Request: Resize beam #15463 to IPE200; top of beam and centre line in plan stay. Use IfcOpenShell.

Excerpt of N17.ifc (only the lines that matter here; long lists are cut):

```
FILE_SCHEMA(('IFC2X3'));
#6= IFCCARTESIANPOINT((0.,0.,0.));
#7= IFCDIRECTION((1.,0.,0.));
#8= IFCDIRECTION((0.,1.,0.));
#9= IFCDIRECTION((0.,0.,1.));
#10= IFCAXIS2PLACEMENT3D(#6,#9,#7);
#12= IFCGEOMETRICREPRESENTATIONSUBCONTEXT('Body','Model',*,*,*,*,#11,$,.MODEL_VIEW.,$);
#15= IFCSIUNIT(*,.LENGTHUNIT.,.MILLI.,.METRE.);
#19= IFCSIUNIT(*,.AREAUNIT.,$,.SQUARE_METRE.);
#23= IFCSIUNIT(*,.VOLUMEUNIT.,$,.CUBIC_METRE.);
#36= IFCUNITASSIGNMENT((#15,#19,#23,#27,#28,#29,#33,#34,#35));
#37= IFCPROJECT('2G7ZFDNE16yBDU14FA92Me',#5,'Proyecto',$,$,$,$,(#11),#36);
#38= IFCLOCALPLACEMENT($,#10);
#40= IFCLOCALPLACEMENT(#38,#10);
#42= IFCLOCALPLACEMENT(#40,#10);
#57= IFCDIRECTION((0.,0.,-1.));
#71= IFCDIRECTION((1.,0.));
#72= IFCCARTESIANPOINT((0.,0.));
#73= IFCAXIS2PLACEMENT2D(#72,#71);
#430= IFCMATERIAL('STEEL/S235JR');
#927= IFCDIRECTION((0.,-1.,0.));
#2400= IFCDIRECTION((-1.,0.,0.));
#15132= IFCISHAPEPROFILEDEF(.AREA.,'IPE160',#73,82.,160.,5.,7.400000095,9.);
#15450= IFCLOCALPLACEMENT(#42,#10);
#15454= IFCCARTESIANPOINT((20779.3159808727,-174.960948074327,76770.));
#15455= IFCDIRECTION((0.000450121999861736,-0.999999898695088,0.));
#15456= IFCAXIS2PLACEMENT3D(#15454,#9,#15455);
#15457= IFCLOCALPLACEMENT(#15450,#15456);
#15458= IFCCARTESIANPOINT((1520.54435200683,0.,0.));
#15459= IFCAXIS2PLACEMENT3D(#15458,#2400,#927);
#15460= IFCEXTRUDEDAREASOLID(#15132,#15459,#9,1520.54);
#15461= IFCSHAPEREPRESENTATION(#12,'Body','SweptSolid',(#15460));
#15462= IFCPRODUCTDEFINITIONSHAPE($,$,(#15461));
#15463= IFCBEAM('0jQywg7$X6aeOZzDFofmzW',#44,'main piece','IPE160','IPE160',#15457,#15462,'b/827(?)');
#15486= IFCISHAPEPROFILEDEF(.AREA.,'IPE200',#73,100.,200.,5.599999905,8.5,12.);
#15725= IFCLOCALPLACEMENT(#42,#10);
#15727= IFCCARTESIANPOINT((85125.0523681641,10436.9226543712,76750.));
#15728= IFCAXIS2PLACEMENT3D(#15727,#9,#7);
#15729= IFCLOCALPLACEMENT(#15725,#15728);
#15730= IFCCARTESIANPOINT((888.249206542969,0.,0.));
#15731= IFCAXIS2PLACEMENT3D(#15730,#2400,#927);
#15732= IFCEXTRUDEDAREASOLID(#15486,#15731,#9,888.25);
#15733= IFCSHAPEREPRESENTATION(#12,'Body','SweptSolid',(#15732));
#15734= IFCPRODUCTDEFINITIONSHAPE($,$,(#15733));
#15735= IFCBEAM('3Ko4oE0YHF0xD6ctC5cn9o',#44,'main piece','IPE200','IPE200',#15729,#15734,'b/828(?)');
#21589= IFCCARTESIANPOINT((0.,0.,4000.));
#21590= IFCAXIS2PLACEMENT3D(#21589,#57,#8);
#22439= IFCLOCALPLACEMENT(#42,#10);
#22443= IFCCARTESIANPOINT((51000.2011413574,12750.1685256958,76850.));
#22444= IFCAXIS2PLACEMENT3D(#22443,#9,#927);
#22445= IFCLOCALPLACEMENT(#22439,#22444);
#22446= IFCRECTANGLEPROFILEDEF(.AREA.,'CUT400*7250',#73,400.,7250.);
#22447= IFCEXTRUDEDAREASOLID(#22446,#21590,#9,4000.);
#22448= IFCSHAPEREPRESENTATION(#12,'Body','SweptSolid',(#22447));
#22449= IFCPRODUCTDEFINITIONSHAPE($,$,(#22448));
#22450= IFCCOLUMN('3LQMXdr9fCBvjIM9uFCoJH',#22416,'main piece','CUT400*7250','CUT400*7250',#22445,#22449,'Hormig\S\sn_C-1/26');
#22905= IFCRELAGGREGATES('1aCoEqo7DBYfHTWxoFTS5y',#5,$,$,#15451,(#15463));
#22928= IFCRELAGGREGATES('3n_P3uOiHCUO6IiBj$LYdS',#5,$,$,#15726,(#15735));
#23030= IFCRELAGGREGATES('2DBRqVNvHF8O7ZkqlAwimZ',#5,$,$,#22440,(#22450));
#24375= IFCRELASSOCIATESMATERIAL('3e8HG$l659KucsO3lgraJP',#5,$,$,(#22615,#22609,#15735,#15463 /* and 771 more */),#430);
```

```python
import ifcopenshell
import ifcopenshell.util.element
import ifcopenshell.util.representation

model = ifcopenshell.open("N17.ifc")

member = model.by_guid("0jQywg7$X6aeOZzDFofmzW")
source = next(p for p in model.by_type("IfcIShapeProfileDef") if p.ProfileName == "IPE200")

body = ifcopenshell.util.representation.get_representation(member, "Model", "Body")
solid = body.Items[0]
old_profile = solid.SweptArea

# Copy the section's sizes but keep this member's own profile position.
profile = ifcopenshell.util.element.copy(model, source)
# Profiles are centred, so shift by half the change in depth to hold the top.
shift = (old_profile.OverallDepth - profile.OverallDepth) / 2
x, y = old_profile.Position.Location.Coordinates
up = (0.0, 1.0)  # upwards, in the solid's own plane
location = model.createIfcCartesianPoint((x + up[0] * shift, y + up[1] * shift))
profile.Position = model.createIfcAxis2Placement2D(location, old_profile.Position.RefDirection)
solid.SweptArea = profile
if not model.get_total_inverses(old_profile):
    ifcopenshell.util.element.remove_deep2(model, old_profile)
member.Description = member.Description.replace("IPE160", "IPE200")
member.ObjectType = member.ObjectType.replace("IPE160", "IPE200")

print(solid.SweptArea)

model.write("N17_edited.ifc")
```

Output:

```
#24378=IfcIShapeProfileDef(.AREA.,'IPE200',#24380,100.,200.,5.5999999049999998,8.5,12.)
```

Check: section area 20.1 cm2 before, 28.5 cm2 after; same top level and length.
